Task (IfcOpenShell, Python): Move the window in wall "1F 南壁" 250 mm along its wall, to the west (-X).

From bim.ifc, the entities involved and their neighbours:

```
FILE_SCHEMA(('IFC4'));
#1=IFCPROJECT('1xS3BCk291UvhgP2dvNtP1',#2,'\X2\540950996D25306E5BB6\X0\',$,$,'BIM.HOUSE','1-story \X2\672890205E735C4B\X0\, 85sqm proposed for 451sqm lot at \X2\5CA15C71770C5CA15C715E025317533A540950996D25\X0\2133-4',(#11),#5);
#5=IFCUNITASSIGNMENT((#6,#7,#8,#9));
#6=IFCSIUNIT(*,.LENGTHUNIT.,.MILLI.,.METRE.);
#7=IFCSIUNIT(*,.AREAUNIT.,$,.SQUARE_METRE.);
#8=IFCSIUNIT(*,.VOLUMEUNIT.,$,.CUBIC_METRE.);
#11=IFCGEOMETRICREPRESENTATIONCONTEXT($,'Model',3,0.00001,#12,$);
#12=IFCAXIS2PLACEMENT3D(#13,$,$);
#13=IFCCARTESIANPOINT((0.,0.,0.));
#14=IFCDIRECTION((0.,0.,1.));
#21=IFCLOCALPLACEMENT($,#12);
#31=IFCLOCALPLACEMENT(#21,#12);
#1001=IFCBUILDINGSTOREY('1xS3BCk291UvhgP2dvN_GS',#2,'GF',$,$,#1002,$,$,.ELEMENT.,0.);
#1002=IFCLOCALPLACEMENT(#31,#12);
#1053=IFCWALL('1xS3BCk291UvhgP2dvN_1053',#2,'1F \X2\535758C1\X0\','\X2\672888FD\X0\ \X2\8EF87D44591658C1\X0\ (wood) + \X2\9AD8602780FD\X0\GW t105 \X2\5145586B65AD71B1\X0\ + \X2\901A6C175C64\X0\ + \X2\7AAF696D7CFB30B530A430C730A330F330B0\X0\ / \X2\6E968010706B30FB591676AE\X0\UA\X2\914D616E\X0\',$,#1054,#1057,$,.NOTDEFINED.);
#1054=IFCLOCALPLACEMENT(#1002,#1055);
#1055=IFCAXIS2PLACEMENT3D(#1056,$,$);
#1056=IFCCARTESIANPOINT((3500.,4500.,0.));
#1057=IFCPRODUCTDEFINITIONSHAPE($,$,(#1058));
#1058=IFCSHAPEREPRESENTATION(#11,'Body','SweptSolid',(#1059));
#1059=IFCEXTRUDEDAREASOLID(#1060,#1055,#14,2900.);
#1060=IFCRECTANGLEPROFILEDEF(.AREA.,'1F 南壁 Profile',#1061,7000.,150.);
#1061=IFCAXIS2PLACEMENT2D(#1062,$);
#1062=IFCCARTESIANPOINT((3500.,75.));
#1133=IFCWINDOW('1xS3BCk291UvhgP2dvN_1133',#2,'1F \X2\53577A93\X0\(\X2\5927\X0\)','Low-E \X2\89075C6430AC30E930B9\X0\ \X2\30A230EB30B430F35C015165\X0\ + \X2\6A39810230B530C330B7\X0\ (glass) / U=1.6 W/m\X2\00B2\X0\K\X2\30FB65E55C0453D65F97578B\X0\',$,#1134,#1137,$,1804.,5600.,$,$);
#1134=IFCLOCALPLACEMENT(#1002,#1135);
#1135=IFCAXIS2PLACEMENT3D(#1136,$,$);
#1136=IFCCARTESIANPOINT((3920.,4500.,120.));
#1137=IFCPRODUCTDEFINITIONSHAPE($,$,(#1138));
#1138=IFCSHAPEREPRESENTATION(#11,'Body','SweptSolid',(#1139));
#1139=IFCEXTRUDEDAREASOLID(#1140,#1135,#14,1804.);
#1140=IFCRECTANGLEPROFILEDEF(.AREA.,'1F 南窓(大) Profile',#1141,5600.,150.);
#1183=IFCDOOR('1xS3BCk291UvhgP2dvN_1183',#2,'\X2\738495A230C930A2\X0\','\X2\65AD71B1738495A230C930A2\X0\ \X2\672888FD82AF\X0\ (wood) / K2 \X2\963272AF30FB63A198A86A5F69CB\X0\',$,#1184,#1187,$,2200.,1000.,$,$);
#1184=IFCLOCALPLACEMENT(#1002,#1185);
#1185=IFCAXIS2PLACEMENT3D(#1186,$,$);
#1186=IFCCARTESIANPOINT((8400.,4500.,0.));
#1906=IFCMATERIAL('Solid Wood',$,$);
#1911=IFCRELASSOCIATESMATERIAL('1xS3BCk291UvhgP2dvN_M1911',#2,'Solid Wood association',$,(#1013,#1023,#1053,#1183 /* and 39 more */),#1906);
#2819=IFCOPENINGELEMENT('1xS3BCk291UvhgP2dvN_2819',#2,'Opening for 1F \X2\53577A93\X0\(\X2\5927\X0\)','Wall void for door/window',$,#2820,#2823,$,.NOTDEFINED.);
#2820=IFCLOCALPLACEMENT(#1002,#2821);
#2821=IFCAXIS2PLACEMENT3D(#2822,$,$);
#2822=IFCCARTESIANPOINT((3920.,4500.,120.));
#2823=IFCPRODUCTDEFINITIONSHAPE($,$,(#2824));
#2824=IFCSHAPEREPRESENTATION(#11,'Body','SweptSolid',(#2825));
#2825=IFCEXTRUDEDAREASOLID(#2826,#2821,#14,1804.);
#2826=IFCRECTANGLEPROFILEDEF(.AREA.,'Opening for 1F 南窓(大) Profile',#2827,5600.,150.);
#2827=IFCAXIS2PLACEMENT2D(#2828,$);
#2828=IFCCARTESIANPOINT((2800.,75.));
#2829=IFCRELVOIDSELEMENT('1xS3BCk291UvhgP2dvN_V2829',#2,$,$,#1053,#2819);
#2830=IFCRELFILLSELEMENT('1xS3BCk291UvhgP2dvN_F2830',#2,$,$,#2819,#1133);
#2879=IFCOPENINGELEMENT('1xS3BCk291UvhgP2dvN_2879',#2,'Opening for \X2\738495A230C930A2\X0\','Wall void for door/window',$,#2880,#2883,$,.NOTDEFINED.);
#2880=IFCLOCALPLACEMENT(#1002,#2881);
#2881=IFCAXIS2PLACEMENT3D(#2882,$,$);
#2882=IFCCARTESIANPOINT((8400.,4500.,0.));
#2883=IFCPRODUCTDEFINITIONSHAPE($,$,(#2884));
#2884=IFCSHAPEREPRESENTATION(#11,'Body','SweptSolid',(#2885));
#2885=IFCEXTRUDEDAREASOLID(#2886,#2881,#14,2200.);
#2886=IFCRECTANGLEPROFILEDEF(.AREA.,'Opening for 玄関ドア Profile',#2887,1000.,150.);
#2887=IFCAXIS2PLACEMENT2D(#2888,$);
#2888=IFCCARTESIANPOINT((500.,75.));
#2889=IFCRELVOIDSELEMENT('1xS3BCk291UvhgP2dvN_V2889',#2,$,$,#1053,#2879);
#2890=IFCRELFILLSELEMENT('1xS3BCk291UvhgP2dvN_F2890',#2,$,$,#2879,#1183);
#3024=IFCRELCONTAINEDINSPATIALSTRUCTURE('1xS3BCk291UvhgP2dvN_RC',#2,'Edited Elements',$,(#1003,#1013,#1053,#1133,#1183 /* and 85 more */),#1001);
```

```python
import ifcopenshell
import ifcopenshell.api.geometry
import ifcopenshell.util.placement
import ifcopenshell.util.unit

model = ifcopenshell.open("bim.ifc")
unit_scale = ifcopenshell.util.unit.calculate_unit_scale(model)

window = model.by_guid("1xS3BCk291UvhgP2dvN_1133")
opening = window.FillsVoids[0].RelatingOpeningElement
wall = opening.VoidsElements[0].RelatingBuildingElement

wall_matrix = ifcopenshell.util.placement.get_local_placement(wall.ObjectPlacement)
shift = wall_matrix[:3, 0] * -0.25 / unit_scale
before = ifcopenshell.util.placement.get_local_placement(window.ObjectPlacement)[:3, 3].copy()

# The window is not placed relative to its opening, so move both.
for product in (opening, window):
    matrix = ifcopenshell.util.placement.get_local_placement(product.ObjectPlacement)
    matrix[:3, 3] += shift
    ifcopenshell.api.geometry.edit_object_placement(model, product=product, matrix=matrix, is_si=False)

after = ifcopenshell.util.placement.get_local_placement(window.ObjectPlacement)[:3, 3]
print("window moved by", (after - before).round(3) + 0.0)

model.write("bim_v2.ifc")
```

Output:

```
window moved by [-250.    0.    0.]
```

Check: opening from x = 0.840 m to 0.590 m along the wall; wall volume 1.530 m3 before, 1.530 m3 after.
